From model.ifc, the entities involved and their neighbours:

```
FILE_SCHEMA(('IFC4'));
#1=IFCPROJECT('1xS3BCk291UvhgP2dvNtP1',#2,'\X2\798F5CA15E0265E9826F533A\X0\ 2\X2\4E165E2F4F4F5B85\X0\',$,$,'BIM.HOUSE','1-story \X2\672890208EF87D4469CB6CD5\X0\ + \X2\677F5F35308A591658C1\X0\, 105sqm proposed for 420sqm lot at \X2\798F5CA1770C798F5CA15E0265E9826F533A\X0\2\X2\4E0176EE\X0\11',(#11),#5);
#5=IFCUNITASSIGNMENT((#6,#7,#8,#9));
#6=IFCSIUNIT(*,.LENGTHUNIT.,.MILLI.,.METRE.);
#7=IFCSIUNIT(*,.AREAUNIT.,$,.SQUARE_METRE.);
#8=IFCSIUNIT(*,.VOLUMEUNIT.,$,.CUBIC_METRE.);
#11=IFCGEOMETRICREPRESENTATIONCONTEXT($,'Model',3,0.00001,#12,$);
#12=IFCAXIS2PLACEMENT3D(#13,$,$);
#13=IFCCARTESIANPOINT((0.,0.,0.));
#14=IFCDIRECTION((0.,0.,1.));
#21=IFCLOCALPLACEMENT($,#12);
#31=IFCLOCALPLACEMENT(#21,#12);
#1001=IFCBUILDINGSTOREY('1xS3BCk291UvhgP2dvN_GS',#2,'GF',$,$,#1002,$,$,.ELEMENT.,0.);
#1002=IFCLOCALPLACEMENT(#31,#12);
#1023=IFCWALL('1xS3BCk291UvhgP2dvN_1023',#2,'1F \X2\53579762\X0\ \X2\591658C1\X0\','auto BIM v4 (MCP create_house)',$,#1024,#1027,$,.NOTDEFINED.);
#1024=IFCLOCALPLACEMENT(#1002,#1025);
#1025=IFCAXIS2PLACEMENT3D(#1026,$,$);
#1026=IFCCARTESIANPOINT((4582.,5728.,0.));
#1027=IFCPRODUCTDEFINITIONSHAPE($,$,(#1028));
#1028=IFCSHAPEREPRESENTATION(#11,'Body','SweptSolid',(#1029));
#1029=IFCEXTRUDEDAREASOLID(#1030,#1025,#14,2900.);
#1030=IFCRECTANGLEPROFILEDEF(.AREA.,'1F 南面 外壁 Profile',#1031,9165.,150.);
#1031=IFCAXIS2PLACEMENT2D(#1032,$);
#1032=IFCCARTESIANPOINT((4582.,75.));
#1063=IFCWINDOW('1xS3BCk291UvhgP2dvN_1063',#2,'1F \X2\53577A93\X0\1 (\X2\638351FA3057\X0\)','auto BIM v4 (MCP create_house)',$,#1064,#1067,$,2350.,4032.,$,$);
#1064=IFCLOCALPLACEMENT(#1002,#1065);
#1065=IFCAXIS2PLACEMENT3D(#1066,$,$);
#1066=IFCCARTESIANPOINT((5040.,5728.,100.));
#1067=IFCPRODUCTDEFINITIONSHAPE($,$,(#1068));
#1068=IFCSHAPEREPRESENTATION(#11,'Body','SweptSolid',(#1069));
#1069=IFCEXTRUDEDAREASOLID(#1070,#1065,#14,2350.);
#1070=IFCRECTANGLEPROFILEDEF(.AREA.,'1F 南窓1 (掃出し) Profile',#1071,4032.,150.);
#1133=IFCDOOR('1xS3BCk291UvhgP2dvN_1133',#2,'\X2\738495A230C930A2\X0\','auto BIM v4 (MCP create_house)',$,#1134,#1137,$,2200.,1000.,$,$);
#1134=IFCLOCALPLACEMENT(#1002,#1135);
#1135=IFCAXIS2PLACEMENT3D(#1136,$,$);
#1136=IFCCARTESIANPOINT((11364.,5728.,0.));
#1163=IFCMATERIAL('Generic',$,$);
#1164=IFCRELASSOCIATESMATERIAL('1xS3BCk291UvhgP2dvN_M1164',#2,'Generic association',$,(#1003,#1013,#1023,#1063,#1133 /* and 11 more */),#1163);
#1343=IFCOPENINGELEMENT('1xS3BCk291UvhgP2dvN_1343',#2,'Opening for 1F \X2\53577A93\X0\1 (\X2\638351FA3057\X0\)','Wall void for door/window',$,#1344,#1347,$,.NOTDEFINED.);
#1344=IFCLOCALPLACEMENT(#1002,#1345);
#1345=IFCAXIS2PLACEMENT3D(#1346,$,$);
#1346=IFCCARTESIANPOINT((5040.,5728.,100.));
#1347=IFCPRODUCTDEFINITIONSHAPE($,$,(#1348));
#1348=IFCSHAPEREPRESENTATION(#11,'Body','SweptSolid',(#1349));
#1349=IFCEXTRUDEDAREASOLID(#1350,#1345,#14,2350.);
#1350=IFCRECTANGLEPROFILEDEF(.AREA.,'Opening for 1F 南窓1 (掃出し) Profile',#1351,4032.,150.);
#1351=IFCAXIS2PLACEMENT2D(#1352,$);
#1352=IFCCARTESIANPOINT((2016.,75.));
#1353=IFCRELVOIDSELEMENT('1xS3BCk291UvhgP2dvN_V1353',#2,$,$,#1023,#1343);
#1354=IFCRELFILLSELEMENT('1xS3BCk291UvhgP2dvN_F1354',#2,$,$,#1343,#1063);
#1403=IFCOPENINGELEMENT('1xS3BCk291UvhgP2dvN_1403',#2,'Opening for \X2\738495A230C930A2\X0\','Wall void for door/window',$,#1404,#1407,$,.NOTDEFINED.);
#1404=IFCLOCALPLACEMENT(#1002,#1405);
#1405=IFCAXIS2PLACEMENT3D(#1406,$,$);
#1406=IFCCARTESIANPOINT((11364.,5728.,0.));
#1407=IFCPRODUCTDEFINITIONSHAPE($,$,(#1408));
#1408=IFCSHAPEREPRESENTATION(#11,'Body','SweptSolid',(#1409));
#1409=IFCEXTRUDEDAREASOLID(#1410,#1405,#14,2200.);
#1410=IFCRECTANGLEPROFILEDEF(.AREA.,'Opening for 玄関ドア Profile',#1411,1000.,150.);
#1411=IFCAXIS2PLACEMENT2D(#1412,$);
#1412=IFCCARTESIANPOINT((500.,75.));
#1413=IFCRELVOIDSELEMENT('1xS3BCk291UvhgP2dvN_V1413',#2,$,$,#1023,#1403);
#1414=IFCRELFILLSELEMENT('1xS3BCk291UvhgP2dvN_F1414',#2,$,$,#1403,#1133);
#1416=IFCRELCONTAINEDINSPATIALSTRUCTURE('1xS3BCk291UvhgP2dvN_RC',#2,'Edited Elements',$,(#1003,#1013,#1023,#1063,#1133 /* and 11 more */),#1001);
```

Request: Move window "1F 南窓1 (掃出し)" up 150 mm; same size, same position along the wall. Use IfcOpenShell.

```python
import numpy as np
import ifcopenshell
import ifcopenshell.api.geometry
import ifcopenshell.util.placement
import ifcopenshell.util.unit

model = ifcopenshell.open("model.ifc")
unit_scale = ifcopenshell.util.unit.calculate_unit_scale(model)

window = model.by_guid("1xS3BCk291UvhgP2dvN_1063")
opening = window.FillsVoids[0].RelatingOpeningElement
dz = 0.15 / unit_scale

shift = np.array([0.0, 0.0, dz])
# The window is not placed relative to its opening, so move both.
for product in (opening, window):
    matrix = ifcopenshell.util.placement.get_local_placement(product.ObjectPlacement)
    matrix[:3, 3] += shift
    ifcopenshell.api.geometry.edit_object_placement(model, product=product, matrix=matrix, is_si=False)

print(f"moved by {dz * unit_scale:+.3f} m")

model.write("model_updated.ifc")
```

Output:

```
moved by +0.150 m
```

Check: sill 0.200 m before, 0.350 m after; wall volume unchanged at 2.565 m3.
